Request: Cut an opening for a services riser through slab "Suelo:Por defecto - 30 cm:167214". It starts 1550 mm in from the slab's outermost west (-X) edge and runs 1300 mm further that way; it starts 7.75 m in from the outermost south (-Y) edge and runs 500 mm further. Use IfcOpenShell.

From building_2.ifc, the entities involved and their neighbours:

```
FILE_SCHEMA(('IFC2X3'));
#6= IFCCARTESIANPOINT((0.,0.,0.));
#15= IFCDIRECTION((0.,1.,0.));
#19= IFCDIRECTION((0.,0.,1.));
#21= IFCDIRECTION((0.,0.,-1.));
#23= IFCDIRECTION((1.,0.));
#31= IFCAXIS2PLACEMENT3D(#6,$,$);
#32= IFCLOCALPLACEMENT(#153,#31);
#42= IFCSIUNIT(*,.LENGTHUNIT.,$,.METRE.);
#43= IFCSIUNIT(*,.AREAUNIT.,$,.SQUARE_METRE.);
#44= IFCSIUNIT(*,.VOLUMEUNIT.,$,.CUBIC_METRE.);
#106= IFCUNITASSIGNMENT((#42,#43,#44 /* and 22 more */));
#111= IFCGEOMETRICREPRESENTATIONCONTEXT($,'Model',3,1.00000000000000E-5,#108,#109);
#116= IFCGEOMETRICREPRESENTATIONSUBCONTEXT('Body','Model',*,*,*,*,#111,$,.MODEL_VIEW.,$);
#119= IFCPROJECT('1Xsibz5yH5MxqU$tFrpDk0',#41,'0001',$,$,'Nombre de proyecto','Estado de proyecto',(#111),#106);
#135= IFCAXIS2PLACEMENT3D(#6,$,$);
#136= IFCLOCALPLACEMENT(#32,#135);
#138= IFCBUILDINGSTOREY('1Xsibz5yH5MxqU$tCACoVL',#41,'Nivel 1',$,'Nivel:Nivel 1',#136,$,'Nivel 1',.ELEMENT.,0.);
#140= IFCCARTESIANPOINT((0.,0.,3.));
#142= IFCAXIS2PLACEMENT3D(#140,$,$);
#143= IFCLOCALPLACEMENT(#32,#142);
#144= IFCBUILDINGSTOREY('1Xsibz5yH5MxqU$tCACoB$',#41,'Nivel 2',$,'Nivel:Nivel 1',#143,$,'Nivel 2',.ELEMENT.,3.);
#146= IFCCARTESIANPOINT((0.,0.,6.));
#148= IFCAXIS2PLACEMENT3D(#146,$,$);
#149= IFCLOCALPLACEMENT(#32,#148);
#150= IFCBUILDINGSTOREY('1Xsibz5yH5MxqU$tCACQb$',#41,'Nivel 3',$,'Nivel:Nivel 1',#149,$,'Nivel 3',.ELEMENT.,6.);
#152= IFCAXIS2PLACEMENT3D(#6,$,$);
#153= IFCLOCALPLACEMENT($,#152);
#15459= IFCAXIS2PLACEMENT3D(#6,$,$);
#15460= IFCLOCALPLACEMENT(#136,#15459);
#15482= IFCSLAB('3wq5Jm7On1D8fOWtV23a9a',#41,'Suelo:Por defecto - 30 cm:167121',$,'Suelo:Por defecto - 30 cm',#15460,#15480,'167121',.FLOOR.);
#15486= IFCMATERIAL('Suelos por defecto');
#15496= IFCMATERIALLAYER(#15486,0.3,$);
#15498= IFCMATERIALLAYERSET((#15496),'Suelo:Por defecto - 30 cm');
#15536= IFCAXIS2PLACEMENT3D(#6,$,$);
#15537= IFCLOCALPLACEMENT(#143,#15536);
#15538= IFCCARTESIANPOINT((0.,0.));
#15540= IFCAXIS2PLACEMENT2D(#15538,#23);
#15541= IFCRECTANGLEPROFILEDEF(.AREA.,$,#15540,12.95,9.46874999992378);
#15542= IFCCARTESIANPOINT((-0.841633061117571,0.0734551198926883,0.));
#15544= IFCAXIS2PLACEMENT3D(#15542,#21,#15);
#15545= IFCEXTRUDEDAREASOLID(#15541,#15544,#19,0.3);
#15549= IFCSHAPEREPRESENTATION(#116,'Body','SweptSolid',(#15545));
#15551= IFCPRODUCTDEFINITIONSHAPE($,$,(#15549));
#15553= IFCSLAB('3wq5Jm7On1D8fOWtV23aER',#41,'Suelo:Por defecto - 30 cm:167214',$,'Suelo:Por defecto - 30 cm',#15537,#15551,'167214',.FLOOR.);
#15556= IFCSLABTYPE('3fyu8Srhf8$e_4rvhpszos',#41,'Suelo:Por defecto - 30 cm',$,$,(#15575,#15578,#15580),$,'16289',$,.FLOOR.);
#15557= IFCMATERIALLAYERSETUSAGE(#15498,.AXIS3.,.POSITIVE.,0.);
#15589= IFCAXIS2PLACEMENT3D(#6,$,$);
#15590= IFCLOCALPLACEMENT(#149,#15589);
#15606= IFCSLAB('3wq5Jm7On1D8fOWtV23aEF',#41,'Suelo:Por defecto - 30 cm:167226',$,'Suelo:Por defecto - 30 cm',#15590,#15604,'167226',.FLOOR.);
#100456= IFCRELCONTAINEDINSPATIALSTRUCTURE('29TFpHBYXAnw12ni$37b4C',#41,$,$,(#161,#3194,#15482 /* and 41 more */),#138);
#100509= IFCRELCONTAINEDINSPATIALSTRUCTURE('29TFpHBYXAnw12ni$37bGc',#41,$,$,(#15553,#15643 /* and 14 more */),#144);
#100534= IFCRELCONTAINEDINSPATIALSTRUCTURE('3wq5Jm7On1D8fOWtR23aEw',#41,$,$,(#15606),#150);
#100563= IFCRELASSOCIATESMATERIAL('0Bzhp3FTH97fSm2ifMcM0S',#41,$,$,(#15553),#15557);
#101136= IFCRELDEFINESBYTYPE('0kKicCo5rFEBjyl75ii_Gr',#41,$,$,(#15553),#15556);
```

```python
import numpy as np
import ifcopenshell
import ifcopenshell.api.feature
import ifcopenshell.api.geometry
import ifcopenshell.api.root
import ifcopenshell.geom
import ifcopenshell.util.placement
import ifcopenshell.util.representation
import ifcopenshell.util.shape
import ifcopenshell.util.unit

model = ifcopenshell.open("building_2.ifc")
unit_scale = ifcopenshell.util.unit.calculate_unit_scale(model)
settings = ifcopenshell.geom.settings()


def volume(element):
    """Net volume in cubic metres, openings subtracted."""
    shape = ifcopenshell.geom.create_shape(settings, element)
    return ifcopenshell.util.shape.get_volume(shape.geometry)


slab = model.by_guid("3wq5Jm7On1D8fOWtV23aER")
before = volume(slab)

# Extent in the slab's own axes, in metres. The edges named are its -X and -Y sides.
slab_shape = ifcopenshell.geom.create_shape(settings, slab)
vertices = ifcopenshell.util.shape.get_vertices(slab_shape.geometry)
x_min, y_min, bottom = vertices.min(axis=0)
top = vertices[:, 2].max()

opening = ifcopenshell.api.root.create_entity(model, ifc_class="IfcOpeningElement", name="Services riser opening")
context = ifcopenshell.util.representation.get_context(model, "Model", "Body", "MODEL_VIEW")
width, depth = 1.3, 0.5
outline = [(0.0, 0.0), (width, 0.0), (width, depth), (0.0, depth), (0.0, 0.0)]
# Overshoot both faces by 50 mm so the cut is clean.
shape = ifcopenshell.api.geometry.add_slab_representation(
    model, context=context, depth=top - bottom + 0.1, polyline=outline
)
ifcopenshell.api.geometry.assign_representation(model, product=opening, representation=shape)

matrix = ifcopenshell.util.placement.get_local_placement(slab.ObjectPlacement)
matrix[:, 3] = matrix @ np.append(np.array([x_min + 1.55, y_min + 7.75, bottom - 0.05]) / unit_scale, 1.0)
ifcopenshell.api.geometry.edit_object_placement(model, product=opening, matrix=matrix, is_si=False)
ifcopenshell.api.feature.add_feature(model, feature=opening, element=slab)

after = volume(slab)

print(f"slab volume {before:.3f} -> {after:.3f} m3")

model.write("building_2-out.ifc")
```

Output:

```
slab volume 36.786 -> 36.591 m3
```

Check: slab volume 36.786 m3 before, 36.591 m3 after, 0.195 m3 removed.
